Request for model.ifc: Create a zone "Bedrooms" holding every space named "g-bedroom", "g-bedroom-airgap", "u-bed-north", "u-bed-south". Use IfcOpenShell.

First a look at what the model holds.

```python
import ifcopenshell

model = ifcopenshell.open("model.ifc")
print(model.schema)
seen = {}
for space in model.by_type("IfcSpace"):
    seen[space.LongName] = seen.get(space.LongName, 0) + 1
for name, count in sorted(seen.items(), key=str):
    print(count, "x", name)
print("zones:", [z.Name for z in model.by_type("IfcZone")][:20])
```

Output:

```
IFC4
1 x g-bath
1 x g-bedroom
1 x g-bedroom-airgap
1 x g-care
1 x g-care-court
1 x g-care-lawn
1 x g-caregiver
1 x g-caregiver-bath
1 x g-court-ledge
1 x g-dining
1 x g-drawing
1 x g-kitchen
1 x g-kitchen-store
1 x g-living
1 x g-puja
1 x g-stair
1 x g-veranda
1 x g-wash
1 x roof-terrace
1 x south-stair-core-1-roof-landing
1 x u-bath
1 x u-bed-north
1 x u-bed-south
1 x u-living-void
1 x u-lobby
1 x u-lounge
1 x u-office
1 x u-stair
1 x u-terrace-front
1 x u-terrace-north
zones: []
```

```python
import ifcopenshell
import ifcopenshell.api.group
import ifcopenshell.api.root

model = ifcopenshell.open("model.ifc")

names = {"g-bedroom", "g-bedroom-airgap", "u-bed-north", "u-bed-south"}
spaces = [s for s in model.by_type("IfcSpace") if s.LongName in names]

zone = ifcopenshell.api.root.create_entity(model, ifc_class="IfcZone", name="Bedrooms")
ifcopenshell.api.group.assign_group(model, products=spaces, group=zone)
print(len(spaces), "spaces in", zone.Name)

model.write("model_edited.ifc")
```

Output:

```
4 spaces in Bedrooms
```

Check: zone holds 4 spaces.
